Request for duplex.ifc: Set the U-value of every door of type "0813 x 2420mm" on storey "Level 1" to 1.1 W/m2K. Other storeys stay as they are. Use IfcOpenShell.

First a look at what the model holds.

```python
import ifcopenshell
import ifcopenshell.util.element

model = ifcopenshell.open("duplex.ifc")
print(model.schema)
storey = next(s for s in model.by_type("IfcBuildingStorey") if s.Name == "Level 1")
doors = [e for e in ifcopenshell.util.element.get_decomposition(storey) if e.is_a("IfcDoor")]
seen = {}
for e in doors:
    element_type = ifcopenshell.util.element.get_type(e)
    key = (element_type.Name if element_type != e and element_type else None, ifcopenshell.util.element.get_pset(e, "Pset_DoorCommon", "ThermalTransmittance"))
    seen[key] = seen.get(key, 0) + 1
for (name, value), count in sorted(seen.items(), key=str):
    print(count, "x", name, "|", value)
```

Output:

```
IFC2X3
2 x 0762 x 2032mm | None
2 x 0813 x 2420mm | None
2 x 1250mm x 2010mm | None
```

```python
import ifcopenshell
import ifcopenshell.api.pset
import ifcopenshell.util.element

model = ifcopenshell.open("duplex.ifc")

storey = next(s for s in model.by_type("IfcBuildingStorey") if s.Name == "Level 1")
doors = [e for e in ifcopenshell.util.element.get_decomposition(storey) if e.is_a("IfcDoor")]

count = 0
for e in doors:
    element_type = ifcopenshell.util.element.get_type(e)
    if element_type in (None, e) or element_type.Name != "0813 x 2420mm":
        continue
    # add_pset returns the element's existing set when there is one.
    pset = ifcopenshell.api.pset.add_pset(model, product=e, name="Pset_DoorCommon")
    ifcopenshell.api.pset.edit_pset(model, pset=pset, properties={"ThermalTransmittance": 1.1})
    count += 1

print(count, "doors updated")

model.write("duplex_v2.ifc")
```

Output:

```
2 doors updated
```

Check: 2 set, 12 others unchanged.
